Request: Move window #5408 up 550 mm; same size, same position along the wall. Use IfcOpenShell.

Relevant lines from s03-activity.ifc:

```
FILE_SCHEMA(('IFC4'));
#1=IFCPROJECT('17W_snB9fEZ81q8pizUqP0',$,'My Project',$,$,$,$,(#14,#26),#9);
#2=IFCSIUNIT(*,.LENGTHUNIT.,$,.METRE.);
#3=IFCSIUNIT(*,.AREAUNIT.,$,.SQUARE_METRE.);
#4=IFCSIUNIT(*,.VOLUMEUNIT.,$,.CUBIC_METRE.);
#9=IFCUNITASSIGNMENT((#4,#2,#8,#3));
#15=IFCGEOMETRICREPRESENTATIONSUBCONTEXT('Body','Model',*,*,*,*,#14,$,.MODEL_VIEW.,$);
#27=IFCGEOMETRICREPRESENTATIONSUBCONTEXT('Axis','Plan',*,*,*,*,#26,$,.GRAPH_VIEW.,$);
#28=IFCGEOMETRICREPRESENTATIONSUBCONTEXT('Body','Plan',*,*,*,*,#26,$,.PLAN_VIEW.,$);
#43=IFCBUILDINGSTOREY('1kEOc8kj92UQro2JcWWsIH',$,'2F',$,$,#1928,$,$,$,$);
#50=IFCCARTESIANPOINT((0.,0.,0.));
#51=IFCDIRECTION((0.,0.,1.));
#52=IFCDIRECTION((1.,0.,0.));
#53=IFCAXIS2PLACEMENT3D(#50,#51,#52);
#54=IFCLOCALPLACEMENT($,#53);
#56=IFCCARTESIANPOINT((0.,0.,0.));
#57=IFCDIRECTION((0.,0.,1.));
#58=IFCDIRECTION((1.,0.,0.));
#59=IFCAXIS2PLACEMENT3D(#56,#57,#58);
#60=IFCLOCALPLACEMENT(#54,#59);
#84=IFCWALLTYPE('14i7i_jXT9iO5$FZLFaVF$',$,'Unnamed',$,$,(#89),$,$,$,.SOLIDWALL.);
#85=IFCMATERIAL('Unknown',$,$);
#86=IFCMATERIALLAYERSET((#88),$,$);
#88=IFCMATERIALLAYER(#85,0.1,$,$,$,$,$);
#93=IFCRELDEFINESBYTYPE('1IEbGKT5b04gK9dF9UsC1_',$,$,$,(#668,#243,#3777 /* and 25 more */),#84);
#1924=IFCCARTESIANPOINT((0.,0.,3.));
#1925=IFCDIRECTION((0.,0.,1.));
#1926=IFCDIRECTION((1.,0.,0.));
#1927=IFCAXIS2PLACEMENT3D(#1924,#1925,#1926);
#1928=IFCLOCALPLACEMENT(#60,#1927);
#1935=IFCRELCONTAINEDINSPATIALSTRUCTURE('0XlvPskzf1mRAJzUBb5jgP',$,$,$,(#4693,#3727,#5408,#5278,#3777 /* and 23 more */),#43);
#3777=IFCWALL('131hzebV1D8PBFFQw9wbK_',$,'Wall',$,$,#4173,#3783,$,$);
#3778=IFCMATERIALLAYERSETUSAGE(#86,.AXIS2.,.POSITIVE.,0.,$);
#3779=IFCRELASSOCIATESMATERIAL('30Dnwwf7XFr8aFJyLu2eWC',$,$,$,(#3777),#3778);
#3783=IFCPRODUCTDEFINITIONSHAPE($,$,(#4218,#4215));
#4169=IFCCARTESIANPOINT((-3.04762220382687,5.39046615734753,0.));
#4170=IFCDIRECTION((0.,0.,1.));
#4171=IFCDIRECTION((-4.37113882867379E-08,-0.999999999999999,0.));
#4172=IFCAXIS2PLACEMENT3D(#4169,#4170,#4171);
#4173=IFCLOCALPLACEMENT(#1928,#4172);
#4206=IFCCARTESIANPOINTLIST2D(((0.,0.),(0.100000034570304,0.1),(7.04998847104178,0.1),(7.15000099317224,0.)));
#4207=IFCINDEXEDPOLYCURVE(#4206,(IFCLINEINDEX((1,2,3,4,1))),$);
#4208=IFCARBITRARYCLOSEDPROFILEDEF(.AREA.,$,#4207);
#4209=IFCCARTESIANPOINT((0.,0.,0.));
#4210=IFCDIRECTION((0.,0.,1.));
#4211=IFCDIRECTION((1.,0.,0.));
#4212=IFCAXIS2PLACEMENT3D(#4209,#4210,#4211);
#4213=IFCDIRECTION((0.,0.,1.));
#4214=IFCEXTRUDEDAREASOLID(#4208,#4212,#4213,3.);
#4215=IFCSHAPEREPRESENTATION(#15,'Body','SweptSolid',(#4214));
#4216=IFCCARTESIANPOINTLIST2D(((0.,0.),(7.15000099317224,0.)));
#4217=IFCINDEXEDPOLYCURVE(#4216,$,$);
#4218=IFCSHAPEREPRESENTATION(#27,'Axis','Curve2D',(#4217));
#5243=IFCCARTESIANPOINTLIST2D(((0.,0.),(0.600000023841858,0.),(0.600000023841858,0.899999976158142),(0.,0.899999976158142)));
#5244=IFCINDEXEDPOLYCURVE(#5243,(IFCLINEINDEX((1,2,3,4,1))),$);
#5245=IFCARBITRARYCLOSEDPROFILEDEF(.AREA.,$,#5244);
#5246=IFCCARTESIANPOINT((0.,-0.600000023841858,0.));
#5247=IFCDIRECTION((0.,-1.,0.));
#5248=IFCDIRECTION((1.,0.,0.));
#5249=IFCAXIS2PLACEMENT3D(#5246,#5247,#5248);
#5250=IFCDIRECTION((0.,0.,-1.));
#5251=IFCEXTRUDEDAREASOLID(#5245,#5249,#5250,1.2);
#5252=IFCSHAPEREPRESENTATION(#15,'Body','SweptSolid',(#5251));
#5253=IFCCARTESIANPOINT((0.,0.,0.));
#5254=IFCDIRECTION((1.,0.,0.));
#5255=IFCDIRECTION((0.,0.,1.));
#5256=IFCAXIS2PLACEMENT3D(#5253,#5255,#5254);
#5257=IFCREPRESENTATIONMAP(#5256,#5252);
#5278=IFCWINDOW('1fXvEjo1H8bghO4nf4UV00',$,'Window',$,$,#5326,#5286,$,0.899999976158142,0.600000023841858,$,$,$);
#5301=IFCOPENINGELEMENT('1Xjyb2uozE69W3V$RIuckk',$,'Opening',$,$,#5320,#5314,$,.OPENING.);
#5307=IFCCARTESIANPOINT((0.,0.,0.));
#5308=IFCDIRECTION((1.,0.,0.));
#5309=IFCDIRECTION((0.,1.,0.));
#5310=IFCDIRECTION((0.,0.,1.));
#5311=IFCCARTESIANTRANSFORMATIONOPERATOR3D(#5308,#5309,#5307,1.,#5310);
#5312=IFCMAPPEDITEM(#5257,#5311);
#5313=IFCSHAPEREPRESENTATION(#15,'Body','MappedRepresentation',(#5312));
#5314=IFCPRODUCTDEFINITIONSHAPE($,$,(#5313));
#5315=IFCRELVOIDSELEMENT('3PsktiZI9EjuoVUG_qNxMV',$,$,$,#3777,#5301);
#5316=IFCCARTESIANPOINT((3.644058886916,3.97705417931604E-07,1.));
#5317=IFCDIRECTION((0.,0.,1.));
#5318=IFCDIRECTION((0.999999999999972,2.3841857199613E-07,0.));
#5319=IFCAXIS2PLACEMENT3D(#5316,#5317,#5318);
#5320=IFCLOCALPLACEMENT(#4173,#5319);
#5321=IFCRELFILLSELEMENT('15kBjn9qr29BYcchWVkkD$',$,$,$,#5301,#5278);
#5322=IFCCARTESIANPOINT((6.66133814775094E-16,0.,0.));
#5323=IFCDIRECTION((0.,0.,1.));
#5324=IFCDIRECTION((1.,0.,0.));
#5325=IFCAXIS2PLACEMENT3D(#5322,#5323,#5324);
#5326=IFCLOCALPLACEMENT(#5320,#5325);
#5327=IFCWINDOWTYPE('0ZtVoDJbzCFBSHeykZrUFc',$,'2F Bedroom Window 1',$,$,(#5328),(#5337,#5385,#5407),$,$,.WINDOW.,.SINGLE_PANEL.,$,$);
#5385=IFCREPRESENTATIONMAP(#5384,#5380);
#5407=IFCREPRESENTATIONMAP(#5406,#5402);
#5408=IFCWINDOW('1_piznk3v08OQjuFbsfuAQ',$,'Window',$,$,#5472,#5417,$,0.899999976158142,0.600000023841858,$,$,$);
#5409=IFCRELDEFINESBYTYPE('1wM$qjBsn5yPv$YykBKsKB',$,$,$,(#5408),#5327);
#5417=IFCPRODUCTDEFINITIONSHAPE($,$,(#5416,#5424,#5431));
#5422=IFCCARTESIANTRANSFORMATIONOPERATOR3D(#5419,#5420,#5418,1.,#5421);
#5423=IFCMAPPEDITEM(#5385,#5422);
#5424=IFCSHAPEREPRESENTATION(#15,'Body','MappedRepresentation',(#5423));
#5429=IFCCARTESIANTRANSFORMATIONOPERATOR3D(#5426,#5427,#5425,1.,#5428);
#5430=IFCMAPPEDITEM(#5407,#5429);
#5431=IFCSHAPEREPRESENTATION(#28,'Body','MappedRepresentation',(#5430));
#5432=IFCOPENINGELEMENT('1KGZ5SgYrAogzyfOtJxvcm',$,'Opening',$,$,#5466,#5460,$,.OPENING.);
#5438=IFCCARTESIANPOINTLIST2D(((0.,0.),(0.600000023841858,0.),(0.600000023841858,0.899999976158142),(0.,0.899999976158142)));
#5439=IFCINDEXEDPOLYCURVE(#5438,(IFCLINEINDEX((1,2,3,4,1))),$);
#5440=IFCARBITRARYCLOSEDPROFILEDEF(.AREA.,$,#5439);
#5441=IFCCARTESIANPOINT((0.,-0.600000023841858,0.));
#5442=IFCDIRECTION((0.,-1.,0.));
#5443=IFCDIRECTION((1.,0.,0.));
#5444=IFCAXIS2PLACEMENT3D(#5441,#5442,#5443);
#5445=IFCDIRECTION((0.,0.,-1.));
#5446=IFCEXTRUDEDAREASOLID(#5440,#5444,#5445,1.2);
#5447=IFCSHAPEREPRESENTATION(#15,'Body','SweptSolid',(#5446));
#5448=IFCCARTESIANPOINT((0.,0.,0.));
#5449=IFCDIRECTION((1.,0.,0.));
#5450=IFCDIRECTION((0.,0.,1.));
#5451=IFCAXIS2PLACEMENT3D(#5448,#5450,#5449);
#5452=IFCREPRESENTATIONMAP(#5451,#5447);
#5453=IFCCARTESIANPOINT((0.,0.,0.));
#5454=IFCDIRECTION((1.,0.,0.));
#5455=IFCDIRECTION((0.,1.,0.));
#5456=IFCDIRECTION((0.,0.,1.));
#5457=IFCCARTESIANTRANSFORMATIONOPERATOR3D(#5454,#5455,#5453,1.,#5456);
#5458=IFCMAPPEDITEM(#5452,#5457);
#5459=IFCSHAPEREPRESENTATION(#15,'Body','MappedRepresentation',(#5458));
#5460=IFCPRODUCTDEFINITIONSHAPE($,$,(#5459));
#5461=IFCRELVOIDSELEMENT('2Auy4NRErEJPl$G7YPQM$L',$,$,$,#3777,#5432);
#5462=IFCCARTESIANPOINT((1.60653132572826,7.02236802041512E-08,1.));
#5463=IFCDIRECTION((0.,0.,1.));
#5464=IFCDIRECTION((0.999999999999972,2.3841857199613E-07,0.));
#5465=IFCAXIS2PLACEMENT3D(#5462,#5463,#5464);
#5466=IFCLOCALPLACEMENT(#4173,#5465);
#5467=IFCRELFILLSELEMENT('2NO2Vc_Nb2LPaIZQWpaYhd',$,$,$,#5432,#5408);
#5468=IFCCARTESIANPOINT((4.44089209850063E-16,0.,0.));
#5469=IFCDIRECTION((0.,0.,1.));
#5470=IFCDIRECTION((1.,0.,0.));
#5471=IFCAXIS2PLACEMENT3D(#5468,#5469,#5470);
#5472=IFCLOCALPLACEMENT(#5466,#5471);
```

```python
import numpy as np
import ifcopenshell
import ifcopenshell.api.geometry
import ifcopenshell.util.placement
import ifcopenshell.util.unit

model = ifcopenshell.open("s03-activity.ifc")
unit_scale = ifcopenshell.util.unit.calculate_unit_scale(model)

window = model.by_guid("1_piznk3v08OQjuFbsfuAQ")
opening = window.FillsVoids[0].RelatingOpeningElement
dz = 0.55 / unit_scale

shift = np.array([0.0, 0.0, dz])
# The window is placed relative to its opening, so it follows when the opening moves.
matrix = ifcopenshell.util.placement.get_local_placement(opening.ObjectPlacement)
matrix[:3, 3] += shift
ifcopenshell.api.geometry.edit_object_placement(
    model, product=opening, matrix=matrix, is_si=False, should_transform_children=True
)

print(f"moved by {dz * unit_scale:+.3f} m")

model.write("s03-activity-out.ifc")
```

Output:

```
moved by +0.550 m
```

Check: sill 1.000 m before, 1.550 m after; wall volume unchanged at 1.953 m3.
